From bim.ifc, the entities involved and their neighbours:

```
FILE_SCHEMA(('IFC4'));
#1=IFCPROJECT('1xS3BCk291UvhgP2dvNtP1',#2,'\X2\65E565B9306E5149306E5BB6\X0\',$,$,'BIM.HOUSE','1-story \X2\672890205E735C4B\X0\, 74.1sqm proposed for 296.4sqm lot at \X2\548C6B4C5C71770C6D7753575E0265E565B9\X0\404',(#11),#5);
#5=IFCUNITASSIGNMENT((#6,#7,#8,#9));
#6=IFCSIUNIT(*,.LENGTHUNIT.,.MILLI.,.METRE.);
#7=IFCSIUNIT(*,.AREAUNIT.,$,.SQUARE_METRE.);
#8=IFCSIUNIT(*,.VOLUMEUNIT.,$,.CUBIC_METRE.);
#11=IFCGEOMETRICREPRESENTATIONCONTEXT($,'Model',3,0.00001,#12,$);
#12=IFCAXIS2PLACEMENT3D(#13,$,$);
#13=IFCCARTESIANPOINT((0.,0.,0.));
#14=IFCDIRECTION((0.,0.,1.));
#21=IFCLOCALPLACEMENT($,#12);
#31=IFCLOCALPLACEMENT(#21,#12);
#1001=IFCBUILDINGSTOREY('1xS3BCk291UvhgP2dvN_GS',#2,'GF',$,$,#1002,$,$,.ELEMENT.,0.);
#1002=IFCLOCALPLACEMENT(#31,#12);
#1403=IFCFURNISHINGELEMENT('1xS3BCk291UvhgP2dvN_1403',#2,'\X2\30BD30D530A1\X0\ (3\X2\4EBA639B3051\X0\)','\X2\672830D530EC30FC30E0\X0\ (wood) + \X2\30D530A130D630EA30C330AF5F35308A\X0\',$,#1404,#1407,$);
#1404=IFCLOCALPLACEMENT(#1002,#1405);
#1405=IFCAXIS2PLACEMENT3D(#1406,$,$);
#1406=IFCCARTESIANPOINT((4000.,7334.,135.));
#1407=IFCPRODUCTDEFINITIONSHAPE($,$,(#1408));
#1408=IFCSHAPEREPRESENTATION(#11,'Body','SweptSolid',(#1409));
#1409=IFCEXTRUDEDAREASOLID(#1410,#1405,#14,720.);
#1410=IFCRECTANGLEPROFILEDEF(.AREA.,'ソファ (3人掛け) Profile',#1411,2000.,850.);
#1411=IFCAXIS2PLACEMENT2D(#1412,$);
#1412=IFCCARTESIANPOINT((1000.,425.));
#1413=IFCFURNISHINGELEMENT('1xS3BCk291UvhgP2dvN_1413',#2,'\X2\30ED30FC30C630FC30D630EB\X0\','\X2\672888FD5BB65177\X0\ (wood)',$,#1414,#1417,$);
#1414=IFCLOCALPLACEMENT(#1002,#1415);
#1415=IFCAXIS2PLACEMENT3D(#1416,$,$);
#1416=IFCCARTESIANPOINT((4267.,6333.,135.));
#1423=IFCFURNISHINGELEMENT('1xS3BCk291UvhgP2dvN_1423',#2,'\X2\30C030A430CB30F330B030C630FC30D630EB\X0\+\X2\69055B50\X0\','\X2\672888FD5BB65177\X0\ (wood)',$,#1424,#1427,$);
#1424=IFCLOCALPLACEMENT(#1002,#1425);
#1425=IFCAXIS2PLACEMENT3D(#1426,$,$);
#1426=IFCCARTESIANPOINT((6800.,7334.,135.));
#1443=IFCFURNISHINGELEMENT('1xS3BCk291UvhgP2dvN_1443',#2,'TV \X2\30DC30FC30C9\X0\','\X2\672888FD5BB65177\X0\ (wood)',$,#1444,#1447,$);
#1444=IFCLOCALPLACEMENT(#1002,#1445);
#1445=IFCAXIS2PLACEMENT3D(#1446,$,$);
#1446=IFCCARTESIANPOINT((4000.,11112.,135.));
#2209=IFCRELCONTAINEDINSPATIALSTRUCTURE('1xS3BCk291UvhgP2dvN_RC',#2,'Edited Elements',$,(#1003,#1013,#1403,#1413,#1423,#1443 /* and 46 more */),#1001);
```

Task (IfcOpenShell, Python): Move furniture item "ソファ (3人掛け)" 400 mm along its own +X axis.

```python
import ifcopenshell
import ifcopenshell.api.geometry
import ifcopenshell.util.placement
import ifcopenshell.util.unit

model = ifcopenshell.open("bim.ifc")
unit_scale = ifcopenshell.util.unit.calculate_unit_scale(model)

item = model.by_guid("1xS3BCk291UvhgP2dvN_1403")
matrix = ifcopenshell.util.placement.get_local_placement(item.ObjectPlacement)
matrix[:3, 3] += matrix[:3, 0] * 0.4 / unit_scale
ifcopenshell.api.geometry.edit_object_placement(model, product=item, matrix=matrix, is_si=False)

print(ifcopenshell.util.placement.get_local_placement(item.ObjectPlacement).round(3) + 0.0)

model.write("bim_edited.ifc")
```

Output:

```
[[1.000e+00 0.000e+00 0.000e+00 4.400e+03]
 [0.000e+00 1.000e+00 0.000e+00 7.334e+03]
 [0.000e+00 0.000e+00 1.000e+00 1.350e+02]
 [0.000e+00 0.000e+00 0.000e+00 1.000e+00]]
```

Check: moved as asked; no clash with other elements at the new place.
